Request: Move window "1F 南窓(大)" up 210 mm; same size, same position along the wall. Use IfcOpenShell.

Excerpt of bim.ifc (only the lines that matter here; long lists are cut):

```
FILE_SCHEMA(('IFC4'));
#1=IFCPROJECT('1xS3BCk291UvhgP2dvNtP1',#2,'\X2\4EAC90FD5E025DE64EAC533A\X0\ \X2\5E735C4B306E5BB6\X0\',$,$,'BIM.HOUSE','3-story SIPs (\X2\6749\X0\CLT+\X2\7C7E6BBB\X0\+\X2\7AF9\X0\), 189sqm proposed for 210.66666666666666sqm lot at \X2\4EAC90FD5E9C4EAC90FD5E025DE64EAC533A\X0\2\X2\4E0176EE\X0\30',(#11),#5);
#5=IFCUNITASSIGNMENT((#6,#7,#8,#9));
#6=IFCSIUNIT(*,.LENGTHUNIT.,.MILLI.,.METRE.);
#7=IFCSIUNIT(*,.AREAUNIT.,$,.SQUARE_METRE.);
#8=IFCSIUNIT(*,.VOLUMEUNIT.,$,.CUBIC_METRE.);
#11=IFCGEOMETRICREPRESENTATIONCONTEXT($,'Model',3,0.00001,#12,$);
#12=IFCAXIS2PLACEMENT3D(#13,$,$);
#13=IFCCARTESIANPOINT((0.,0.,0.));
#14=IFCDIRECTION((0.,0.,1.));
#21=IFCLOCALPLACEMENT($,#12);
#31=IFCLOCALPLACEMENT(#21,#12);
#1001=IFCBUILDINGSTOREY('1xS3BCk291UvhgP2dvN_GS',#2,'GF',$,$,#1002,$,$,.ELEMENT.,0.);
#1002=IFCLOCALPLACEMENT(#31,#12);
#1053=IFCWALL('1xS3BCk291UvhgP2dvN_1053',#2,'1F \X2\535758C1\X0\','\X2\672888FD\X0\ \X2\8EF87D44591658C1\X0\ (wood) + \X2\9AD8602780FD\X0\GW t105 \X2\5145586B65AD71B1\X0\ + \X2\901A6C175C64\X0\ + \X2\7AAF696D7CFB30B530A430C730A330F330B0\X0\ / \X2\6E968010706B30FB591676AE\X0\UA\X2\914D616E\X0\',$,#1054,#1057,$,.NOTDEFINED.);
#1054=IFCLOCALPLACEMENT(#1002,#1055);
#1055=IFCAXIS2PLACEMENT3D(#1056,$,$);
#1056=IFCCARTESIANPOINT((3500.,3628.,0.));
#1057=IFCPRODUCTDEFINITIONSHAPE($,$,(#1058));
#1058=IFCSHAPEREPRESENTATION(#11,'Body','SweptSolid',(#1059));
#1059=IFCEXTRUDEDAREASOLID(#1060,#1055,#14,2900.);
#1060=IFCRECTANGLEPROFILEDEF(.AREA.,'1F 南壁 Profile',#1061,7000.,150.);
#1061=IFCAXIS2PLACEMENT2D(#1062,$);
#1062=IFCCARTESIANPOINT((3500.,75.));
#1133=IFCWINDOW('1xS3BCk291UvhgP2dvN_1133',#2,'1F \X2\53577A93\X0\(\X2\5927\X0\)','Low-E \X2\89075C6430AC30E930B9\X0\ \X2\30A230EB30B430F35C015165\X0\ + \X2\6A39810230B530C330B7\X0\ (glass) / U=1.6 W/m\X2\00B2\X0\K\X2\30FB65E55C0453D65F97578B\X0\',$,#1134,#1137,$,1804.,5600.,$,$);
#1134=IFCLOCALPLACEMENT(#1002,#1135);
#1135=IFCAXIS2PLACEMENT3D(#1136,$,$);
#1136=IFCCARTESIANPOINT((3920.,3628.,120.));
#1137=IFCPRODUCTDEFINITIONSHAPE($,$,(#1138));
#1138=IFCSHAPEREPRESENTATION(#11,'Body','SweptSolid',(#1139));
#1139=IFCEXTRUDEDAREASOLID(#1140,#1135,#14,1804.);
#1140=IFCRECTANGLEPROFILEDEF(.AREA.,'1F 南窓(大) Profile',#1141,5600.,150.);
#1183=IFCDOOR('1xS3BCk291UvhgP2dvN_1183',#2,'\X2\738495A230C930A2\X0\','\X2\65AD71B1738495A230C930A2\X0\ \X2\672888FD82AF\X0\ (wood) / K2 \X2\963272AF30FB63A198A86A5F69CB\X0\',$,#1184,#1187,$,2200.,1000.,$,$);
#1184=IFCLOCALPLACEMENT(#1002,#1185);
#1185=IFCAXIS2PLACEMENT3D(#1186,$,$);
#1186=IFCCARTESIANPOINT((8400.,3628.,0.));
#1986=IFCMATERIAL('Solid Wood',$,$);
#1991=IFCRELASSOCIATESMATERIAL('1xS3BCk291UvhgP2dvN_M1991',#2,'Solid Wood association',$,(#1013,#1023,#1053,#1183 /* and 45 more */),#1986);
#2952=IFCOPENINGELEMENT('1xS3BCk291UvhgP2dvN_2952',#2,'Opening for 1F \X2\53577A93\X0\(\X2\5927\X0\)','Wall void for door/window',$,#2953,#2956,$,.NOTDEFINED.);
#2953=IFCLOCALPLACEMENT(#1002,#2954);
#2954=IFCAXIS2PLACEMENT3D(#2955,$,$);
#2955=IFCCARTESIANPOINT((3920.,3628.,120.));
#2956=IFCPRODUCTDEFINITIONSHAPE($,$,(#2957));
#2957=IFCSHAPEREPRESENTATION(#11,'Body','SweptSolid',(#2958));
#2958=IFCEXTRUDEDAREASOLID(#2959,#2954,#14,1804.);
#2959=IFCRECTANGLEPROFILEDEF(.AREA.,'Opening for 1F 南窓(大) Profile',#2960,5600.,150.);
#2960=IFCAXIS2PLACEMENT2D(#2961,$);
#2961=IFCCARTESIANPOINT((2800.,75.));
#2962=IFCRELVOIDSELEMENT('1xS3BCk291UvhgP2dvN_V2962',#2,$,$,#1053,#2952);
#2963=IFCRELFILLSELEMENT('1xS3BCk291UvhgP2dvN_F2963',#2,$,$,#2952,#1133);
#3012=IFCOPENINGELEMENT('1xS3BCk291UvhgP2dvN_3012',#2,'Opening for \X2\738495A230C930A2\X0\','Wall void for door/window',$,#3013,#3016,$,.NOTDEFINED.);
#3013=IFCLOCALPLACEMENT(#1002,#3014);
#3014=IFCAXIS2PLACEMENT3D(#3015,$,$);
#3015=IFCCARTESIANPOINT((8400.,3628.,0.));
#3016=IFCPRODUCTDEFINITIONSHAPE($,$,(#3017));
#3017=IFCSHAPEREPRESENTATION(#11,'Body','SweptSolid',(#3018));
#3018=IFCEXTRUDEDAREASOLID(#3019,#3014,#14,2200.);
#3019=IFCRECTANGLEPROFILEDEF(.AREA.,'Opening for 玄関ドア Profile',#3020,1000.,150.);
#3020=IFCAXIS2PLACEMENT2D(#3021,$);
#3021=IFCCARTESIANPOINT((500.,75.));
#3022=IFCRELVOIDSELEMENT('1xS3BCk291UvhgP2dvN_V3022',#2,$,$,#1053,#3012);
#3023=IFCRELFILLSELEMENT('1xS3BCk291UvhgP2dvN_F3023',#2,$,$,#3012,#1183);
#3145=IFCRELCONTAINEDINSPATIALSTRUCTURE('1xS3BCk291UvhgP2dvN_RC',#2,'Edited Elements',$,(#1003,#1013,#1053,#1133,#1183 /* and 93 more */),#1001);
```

```python
import numpy as np
import ifcopenshell
import ifcopenshell.api.geometry
import ifcopenshell.util.placement
import ifcopenshell.util.unit

model = ifcopenshell.open("bim.ifc")
unit_scale = ifcopenshell.util.unit.calculate_unit_scale(model)

window = model.by_guid("1xS3BCk291UvhgP2dvN_1133")
opening = window.FillsVoids[0].RelatingOpeningElement
dz = 0.21 / unit_scale

shift = np.array([0.0, 0.0, dz])
# The window is not placed relative to its opening, so move both.
for product in (opening, window):
    matrix = ifcopenshell.util.placement.get_local_placement(product.ObjectPlacement)
    matrix[:3, 3] += shift
    ifcopenshell.api.geometry.edit_object_placement(model, product=product, matrix=matrix, is_si=False)

print(f"moved by {dz * unit_scale:+.3f} m")

model.write("bim_updated.ifc")
```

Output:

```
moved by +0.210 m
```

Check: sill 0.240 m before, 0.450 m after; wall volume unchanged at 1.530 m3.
